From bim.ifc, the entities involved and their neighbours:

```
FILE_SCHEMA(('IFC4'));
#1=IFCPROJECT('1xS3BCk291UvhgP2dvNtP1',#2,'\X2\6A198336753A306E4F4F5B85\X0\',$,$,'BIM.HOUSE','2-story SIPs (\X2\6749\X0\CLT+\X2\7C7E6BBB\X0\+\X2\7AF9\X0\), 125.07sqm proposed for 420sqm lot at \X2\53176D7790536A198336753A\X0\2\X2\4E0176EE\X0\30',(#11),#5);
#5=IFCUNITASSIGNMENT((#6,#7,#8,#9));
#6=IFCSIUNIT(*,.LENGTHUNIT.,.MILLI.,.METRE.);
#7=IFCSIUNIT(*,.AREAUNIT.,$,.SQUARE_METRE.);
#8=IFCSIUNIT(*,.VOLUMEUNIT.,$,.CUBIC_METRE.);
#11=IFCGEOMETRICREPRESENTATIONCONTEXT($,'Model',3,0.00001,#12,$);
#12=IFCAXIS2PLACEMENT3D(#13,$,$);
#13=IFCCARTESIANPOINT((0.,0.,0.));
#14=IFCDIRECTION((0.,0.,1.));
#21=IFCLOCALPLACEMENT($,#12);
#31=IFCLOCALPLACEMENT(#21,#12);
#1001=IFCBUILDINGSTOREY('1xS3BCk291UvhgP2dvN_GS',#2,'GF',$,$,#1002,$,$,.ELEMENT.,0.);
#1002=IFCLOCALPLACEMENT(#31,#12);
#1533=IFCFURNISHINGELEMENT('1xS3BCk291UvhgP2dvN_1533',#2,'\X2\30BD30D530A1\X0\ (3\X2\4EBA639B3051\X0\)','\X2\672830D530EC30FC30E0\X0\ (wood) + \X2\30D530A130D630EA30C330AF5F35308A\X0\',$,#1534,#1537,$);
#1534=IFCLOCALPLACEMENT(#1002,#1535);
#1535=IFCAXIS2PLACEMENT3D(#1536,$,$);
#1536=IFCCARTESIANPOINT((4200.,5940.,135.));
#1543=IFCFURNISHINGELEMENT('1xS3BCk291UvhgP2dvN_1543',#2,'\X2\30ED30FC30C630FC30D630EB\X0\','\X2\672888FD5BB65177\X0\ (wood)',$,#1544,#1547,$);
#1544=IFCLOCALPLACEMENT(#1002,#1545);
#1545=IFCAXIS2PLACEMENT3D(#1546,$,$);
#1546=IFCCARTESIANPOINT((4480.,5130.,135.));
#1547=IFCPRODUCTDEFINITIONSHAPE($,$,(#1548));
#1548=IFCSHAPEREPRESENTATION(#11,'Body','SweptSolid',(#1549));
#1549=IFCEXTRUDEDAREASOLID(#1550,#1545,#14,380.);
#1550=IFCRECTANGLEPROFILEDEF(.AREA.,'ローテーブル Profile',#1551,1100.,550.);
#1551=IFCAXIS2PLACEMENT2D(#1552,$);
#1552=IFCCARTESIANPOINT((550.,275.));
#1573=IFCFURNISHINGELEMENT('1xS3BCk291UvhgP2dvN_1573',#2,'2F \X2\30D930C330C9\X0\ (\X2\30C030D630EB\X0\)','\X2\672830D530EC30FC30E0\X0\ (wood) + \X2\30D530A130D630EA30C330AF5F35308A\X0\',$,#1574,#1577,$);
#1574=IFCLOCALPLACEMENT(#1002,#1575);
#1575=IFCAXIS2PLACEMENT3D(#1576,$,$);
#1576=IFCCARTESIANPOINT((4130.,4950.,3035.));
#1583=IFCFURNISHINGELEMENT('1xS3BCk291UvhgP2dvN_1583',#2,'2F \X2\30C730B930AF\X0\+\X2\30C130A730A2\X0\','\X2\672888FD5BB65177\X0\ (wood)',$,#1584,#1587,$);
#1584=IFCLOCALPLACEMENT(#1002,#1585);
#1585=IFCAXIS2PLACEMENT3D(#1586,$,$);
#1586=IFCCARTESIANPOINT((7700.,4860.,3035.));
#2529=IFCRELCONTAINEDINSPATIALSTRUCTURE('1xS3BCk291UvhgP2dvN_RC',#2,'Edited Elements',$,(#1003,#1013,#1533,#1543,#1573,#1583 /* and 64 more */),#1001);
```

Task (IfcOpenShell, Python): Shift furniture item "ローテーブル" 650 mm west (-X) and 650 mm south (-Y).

```python
import ifcopenshell
import ifcopenshell.api.geometry
import ifcopenshell.util.placement
import ifcopenshell.util.unit

model = ifcopenshell.open("bim.ifc")
unit_scale = ifcopenshell.util.unit.calculate_unit_scale(model)

item = model.by_guid("1xS3BCk291UvhgP2dvN_1543")
matrix = ifcopenshell.util.placement.get_local_placement(item.ObjectPlacement)
matrix[0, 3] -= 0.65 / unit_scale
matrix[1, 3] -= 0.65 / unit_scale
ifcopenshell.api.geometry.edit_object_placement(model, product=item, matrix=matrix, is_si=False)

print(ifcopenshell.util.placement.get_local_placement(item.ObjectPlacement).round(3) + 0.0)

model.write("bim-out.ifc")
```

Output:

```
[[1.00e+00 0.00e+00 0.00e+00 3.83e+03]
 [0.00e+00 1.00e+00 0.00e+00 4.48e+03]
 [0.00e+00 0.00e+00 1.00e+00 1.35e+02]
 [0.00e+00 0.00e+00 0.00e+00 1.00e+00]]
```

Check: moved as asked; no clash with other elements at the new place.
